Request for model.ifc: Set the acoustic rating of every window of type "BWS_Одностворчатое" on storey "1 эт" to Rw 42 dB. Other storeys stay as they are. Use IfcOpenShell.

First a look at what the model holds.

```python
import ifcopenshell
import ifcopenshell.util.element

model = ifcopenshell.open("model.ifc")
print(model.schema)
storey = next(s for s in model.by_type("IfcBuildingStorey") if s.Name == "1 эт")
windows = [e for e in ifcopenshell.util.element.get_decomposition(storey) if e.is_a("IfcWindow")]
seen = {}
for e in windows:
    element_type = ifcopenshell.util.element.get_type(e)
    key = (element_type.Name if element_type != e and element_type else None, ifcopenshell.util.element.get_pset(e, "Pset_WindowCommon", "AcousticRating"))
    seen[key] = seen.get(key, 0) + 1
for (name, value), count in sorted(seen.items(), key=str):
    print(count, "x", name, "|", value)
```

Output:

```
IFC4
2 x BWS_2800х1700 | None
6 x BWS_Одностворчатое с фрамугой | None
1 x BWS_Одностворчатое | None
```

```python
import ifcopenshell
import ifcopenshell.api.pset
import ifcopenshell.util.element

model = ifcopenshell.open("model.ifc")

storey = next(s for s in model.by_type("IfcBuildingStorey") if s.Name == "1 эт")
windows = [e for e in ifcopenshell.util.element.get_decomposition(storey) if e.is_a("IfcWindow")]

count = 0
for e in windows:
    element_type = ifcopenshell.util.element.get_type(e)
    if element_type in (None, e) or element_type.Name != "BWS_Одностворчатое":
        continue
    # add_pset returns the element's existing set when there is one.
    pset = ifcopenshell.api.pset.add_pset(model, product=e, name="Pset_WindowCommon")
    ifcopenshell.api.pset.edit_pset(model, pset=pset, properties={"AcousticRating": "Rw 42 dB"})
    count += 1

print(count, "windows updated")

model.write("model_v2.ifc")
```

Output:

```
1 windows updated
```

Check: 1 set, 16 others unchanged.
